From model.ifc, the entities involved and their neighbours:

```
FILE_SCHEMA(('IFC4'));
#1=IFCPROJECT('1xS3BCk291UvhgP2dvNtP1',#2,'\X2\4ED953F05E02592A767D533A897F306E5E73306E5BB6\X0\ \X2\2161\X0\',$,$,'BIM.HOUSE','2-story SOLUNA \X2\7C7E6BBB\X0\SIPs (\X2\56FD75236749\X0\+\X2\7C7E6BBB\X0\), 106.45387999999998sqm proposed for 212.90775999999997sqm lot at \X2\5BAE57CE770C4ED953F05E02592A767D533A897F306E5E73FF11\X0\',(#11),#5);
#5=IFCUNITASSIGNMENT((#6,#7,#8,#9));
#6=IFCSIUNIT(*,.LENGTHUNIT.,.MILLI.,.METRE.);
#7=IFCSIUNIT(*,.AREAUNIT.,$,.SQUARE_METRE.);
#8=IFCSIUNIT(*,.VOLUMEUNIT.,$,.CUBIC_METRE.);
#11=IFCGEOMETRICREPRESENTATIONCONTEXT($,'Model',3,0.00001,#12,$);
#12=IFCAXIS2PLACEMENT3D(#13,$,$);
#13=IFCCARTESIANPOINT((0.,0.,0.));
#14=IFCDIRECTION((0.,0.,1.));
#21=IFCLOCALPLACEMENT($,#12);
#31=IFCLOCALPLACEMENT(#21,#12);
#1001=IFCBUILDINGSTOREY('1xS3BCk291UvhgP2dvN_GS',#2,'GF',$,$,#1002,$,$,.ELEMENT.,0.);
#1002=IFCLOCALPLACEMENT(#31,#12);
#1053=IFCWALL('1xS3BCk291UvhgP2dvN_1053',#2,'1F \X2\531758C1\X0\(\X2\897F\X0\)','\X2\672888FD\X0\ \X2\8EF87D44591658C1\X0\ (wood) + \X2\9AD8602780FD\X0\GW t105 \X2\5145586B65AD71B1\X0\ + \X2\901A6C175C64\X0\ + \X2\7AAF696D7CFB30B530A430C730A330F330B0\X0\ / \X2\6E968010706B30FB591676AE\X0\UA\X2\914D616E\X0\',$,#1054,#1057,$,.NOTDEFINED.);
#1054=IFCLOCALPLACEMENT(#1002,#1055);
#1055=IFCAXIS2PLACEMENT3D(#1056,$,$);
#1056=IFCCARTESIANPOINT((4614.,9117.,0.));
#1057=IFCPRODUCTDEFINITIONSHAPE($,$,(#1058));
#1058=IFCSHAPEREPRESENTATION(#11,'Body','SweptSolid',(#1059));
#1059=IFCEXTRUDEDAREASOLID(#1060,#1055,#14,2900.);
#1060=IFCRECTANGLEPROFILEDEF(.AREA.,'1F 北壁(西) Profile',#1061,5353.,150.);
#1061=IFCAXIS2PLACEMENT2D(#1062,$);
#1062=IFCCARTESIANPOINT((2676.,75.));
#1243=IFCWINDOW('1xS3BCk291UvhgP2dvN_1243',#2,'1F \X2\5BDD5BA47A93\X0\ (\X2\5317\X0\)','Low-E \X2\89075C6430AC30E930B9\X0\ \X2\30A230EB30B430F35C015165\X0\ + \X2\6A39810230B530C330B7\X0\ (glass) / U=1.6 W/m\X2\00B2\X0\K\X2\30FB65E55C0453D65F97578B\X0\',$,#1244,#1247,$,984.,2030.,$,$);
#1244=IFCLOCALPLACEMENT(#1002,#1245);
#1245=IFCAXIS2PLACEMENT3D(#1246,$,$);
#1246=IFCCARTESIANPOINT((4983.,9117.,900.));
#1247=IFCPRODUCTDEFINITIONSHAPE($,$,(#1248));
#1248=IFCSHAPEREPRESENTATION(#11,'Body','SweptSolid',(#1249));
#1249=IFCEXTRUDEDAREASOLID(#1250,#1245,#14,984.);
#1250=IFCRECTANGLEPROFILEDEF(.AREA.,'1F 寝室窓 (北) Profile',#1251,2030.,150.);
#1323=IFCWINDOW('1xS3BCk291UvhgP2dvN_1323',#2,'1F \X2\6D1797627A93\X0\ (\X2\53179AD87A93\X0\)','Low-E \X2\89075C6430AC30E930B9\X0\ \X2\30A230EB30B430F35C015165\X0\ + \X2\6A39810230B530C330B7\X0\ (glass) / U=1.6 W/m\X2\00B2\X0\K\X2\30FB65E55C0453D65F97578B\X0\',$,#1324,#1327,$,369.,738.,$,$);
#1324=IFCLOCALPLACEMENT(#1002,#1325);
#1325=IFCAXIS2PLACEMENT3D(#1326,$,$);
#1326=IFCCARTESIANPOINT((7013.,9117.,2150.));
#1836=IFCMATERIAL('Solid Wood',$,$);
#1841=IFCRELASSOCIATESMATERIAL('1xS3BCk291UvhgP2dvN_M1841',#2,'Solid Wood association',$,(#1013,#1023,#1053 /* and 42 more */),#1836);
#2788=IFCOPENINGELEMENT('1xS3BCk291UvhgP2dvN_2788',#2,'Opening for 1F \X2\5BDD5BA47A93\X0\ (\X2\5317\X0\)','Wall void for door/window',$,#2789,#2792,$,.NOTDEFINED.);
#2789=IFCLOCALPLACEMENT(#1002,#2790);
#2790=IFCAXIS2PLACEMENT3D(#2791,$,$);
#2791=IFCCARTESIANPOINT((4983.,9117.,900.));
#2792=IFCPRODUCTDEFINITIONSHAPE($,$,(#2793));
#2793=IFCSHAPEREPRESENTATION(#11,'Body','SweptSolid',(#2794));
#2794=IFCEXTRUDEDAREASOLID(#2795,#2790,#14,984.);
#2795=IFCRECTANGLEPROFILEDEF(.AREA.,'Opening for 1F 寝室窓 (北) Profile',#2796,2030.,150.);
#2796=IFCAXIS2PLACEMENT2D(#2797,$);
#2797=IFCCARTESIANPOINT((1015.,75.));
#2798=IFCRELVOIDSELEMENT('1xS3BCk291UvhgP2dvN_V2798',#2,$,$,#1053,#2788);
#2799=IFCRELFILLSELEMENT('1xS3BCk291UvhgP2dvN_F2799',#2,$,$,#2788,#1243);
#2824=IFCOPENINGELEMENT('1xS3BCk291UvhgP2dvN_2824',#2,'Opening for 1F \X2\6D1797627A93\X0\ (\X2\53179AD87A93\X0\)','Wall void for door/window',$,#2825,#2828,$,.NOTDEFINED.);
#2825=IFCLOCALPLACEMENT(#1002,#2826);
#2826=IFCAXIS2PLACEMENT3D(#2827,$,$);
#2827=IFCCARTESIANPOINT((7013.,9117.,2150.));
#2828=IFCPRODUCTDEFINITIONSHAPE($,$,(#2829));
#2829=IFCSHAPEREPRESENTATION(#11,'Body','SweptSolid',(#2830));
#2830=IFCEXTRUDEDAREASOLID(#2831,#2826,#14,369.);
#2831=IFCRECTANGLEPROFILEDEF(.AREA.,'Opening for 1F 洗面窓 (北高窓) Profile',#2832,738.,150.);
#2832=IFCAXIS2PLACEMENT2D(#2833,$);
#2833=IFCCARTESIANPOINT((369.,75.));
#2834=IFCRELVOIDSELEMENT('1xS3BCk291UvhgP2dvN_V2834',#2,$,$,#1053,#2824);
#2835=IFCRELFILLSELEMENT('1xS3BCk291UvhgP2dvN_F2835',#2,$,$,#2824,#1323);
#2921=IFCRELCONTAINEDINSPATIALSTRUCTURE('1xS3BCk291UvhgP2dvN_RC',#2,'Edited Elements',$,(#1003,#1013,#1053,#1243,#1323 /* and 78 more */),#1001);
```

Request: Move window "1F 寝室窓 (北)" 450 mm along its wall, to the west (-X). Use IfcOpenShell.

```python
import ifcopenshell
import ifcopenshell.api.geometry
import ifcopenshell.util.placement
import ifcopenshell.util.unit

model = ifcopenshell.open("model.ifc")
unit_scale = ifcopenshell.util.unit.calculate_unit_scale(model)

window = model.by_guid("1xS3BCk291UvhgP2dvN_1243")
opening = window.FillsVoids[0].RelatingOpeningElement
wall = opening.VoidsElements[0].RelatingBuildingElement

wall_matrix = ifcopenshell.util.placement.get_local_placement(wall.ObjectPlacement)
shift = wall_matrix[:3, 0] * -0.45 / unit_scale
before = ifcopenshell.util.placement.get_local_placement(window.ObjectPlacement)[:3, 3].copy()

# The window is not placed relative to its opening, so move both.
for product in (opening, window):
    matrix = ifcopenshell.util.placement.get_local_placement(product.ObjectPlacement)
    matrix[:3, 3] += shift
    ifcopenshell.api.geometry.edit_object_placement(model, product=product, matrix=matrix, is_si=False)

after = ifcopenshell.util.placement.get_local_placement(window.ObjectPlacement)[:3, 3]
print("window moved by", (after - before).round(3) + 0.0)

model.write("model_v2.ifc")
```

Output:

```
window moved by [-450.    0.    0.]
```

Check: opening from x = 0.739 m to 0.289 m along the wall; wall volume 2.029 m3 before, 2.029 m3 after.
